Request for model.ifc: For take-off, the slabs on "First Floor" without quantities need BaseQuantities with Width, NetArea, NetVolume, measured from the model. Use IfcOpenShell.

First a look at what the model holds.

```python
import ifcopenshell
import ifcopenshell.util.element
import ifcopenshell.util.unit

model = ifcopenshell.open("model.ifc")
print(model.schema)
for unit_type in ("LENGTHUNIT", "AREAUNIT", "VOLUMEUNIT"):
    print(unit_type, ifcopenshell.util.unit.calculate_unit_scale(model, unit_type))
storey = next(s for s in model.by_type("IfcBuildingStorey") if s.Name == "First Floor")
slabs = [e for e in ifcopenshell.util.element.get_decomposition(storey) if e.is_a("IfcSlab")]
for e in sorted(slabs, key=lambda e: e.id()):
    print(e.id(), e.is_a(), e.Name, list(ifcopenshell.util.element.get_psets(e, qtos_only=True)), sep=" | ")
```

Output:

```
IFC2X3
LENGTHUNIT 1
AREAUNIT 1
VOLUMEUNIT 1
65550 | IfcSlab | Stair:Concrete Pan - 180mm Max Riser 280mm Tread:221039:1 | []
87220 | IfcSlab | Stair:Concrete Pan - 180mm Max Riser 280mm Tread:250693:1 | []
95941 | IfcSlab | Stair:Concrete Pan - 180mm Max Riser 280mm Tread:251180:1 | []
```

```python
import ifcopenshell
import ifcopenshell.api.pset
import ifcopenshell.geom
import ifcopenshell.util.element
import ifcopenshell.util.shape
import ifcopenshell.util.unit

model = ifcopenshell.open("model.ifc")
unit_scale = ifcopenshell.util.unit.calculate_unit_scale(model)
area_scale = ifcopenshell.util.unit.calculate_unit_scale(model, "AREAUNIT")
volume_scale = ifcopenshell.util.unit.calculate_unit_scale(model, "VOLUMEUNIT")
settings = ifcopenshell.geom.settings()

storey = next(s for s in model.by_type("IfcBuildingStorey") if s.Name == "First Floor")
slabs = [e for e in ifcopenshell.util.element.get_decomposition(storey) if e.is_a("IfcSlab")]

for e in sorted(slabs, key=lambda e: e.id()):
    if ifcopenshell.util.element.get_psets(e, qtos_only=True, should_inherit=False):
        continue
    # Geometry comes back in metres, in the element's own axes.
    shape = ifcopenshell.geom.create_shape(settings, e)
    values = {
        "Width": ifcopenshell.util.shape.get_z(shape.geometry) / unit_scale,
        "NetArea": ifcopenshell.util.shape.get_footprint_area(shape.geometry) / area_scale,
        "NetVolume": ifcopenshell.util.shape.get_volume(shape.geometry) / volume_scale,
    }
    qto = ifcopenshell.api.pset.add_qto(model, product=e, name="BaseQuantities")
    ifcopenshell.api.pset.edit_qto(model, qto=qto, properties=values)
    print(e.id(), {k: round(v, 3) for k, v in values.items()})

model.write("model-out.ifc")
```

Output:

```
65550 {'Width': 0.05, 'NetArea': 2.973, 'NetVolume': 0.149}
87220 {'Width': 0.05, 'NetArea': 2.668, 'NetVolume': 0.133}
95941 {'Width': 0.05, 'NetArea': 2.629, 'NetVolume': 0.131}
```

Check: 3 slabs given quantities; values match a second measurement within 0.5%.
